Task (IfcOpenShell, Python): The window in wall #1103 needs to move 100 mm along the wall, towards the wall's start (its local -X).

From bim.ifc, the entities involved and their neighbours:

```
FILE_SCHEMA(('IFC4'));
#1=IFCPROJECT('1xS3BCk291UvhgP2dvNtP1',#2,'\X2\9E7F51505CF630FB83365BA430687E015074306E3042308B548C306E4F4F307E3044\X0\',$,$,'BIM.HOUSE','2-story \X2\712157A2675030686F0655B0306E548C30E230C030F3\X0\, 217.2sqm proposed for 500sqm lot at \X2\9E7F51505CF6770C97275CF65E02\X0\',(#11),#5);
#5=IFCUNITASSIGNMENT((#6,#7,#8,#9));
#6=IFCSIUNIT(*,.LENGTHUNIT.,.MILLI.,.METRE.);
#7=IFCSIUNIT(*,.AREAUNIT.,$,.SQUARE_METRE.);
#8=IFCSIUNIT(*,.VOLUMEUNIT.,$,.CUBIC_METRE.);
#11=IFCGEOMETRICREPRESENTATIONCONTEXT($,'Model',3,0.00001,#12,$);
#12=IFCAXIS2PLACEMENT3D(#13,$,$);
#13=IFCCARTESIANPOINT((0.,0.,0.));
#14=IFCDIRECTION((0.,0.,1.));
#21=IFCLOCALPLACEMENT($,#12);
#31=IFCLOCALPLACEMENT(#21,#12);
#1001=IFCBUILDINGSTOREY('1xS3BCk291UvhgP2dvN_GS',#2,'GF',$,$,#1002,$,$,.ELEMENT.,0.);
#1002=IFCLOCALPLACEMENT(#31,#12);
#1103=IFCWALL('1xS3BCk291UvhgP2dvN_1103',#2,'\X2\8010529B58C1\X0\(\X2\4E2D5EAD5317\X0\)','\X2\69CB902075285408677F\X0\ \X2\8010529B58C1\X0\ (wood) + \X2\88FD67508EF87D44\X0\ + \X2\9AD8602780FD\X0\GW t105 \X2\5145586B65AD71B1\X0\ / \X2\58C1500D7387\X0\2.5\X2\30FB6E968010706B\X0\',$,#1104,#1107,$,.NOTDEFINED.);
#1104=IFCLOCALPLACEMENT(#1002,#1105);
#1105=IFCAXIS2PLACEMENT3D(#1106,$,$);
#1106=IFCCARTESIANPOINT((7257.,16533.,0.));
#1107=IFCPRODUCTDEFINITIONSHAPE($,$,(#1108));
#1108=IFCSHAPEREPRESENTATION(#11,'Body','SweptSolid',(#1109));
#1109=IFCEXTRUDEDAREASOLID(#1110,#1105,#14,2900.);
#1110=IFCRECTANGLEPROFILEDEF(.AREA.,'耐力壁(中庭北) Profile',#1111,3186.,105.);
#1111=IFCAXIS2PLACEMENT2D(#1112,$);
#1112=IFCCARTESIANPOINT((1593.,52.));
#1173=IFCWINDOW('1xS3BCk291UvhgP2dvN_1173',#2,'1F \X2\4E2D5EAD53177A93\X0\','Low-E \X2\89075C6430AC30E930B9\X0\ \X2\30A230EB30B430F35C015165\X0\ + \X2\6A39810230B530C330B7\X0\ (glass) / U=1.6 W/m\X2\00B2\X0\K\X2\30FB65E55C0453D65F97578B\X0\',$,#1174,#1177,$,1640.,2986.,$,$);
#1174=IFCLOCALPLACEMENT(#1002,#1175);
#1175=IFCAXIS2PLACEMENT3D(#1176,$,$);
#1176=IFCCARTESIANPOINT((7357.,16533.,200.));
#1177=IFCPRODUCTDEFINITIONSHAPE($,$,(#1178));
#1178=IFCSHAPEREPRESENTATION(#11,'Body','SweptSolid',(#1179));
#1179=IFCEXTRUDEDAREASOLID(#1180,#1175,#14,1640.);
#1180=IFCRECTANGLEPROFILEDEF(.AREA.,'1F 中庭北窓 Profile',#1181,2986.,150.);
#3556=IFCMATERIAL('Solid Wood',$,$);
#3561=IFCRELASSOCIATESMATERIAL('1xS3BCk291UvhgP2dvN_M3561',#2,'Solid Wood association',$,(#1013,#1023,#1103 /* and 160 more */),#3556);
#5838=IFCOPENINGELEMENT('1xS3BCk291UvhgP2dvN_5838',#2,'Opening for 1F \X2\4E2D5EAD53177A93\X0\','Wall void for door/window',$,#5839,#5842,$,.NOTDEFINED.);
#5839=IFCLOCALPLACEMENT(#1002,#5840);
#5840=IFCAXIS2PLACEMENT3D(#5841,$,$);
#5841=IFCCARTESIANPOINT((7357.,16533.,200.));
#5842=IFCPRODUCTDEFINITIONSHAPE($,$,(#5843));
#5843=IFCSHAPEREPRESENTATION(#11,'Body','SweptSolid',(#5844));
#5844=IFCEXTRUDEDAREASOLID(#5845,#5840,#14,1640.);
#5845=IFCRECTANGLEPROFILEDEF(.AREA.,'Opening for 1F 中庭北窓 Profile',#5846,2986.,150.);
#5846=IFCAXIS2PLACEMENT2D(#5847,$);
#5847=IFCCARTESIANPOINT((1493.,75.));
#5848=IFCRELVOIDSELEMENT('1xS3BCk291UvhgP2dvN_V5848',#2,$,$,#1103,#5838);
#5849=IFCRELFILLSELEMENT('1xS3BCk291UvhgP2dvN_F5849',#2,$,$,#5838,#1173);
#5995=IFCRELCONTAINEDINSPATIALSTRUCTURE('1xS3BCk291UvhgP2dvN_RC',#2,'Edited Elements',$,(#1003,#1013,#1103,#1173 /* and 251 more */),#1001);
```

```python
import ifcopenshell
import ifcopenshell.api.geometry
import ifcopenshell.util.placement

model = ifcopenshell.open("bim.ifc")

window = model.by_id(1173)
opening = window.FillsVoids[0].RelatingOpeningElement
wall = opening.VoidsElements[0].RelatingBuildingElement

wall_matrix = ifcopenshell.util.placement.get_local_placement(wall.ObjectPlacement)
shift = wall_matrix[:3, 0] * -100.0
before = ifcopenshell.util.placement.get_local_placement(window.ObjectPlacement)[:3, 3].copy()

# The window is not placed relative to its opening, so move both.
for product in (opening, window):
    matrix = ifcopenshell.util.placement.get_local_placement(product.ObjectPlacement)
    matrix[:3, 3] += shift
    ifcopenshell.api.geometry.edit_object_placement(model, product=product, matrix=matrix, is_si=False)

after = ifcopenshell.util.placement.get_local_placement(window.ObjectPlacement)[:3, 3]
print("window moved by", (after - before).round(3) + 0.0)

model.write("bim_v2.ifc")
```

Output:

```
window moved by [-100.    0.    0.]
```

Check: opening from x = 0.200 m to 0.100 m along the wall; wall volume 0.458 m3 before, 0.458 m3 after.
